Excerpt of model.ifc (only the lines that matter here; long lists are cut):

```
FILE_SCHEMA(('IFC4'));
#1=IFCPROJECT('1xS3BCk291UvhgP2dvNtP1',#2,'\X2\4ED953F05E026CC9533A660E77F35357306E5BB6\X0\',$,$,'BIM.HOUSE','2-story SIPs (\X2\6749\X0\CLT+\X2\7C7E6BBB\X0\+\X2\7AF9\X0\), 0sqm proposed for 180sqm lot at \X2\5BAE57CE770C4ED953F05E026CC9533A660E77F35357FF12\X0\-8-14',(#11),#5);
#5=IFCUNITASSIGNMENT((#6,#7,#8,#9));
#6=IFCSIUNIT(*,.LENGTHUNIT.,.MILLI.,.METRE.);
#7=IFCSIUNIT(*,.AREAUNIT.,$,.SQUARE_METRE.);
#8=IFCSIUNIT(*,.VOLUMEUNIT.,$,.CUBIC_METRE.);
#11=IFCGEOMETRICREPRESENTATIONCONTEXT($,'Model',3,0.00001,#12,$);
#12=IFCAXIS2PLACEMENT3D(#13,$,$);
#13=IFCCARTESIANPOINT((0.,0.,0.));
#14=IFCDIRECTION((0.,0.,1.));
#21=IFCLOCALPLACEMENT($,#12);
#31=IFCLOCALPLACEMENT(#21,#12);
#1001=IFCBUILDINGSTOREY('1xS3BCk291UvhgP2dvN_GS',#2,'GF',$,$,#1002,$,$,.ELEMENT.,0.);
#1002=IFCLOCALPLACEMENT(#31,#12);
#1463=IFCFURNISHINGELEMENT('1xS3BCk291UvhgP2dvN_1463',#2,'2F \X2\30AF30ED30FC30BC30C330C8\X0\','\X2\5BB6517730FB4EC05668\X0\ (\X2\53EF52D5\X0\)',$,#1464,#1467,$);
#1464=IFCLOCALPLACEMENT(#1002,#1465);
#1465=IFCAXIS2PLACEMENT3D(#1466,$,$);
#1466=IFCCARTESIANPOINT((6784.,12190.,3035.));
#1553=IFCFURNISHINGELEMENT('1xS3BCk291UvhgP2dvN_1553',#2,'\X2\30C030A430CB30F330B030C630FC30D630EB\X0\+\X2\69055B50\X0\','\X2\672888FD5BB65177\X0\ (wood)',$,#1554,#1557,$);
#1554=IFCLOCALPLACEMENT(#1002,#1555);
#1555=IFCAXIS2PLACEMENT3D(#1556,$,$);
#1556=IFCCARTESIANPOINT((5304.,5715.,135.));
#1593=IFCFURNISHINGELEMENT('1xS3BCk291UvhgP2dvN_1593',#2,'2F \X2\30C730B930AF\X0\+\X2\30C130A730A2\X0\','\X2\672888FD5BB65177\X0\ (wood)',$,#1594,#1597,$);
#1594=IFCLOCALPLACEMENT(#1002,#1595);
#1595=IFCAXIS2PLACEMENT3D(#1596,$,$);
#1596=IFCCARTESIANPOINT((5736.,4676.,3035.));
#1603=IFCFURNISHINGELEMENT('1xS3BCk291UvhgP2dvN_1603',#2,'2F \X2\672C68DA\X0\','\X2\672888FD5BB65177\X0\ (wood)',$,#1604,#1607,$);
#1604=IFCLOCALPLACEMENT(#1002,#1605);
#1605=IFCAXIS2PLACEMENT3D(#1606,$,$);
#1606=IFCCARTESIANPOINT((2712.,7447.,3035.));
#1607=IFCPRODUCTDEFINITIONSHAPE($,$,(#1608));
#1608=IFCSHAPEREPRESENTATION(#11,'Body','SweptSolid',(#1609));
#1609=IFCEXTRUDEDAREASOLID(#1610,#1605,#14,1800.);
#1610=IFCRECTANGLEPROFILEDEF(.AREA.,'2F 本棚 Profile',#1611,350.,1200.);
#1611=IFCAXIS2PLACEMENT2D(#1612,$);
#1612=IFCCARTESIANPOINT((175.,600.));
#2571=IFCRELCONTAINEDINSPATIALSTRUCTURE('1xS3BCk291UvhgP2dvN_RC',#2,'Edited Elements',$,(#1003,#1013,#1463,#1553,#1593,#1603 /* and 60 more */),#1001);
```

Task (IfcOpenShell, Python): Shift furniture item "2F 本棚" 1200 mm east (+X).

```python
import ifcopenshell
import ifcopenshell.api.geometry
import ifcopenshell.util.placement
import ifcopenshell.util.unit

model = ifcopenshell.open("model.ifc")
unit_scale = ifcopenshell.util.unit.calculate_unit_scale(model)

item = model.by_guid("1xS3BCk291UvhgP2dvN_1603")
matrix = ifcopenshell.util.placement.get_local_placement(item.ObjectPlacement)
matrix[0, 3] += 1.2 / unit_scale
ifcopenshell.api.geometry.edit_object_placement(model, product=item, matrix=matrix, is_si=False)

print(ifcopenshell.util.placement.get_local_placement(item.ObjectPlacement).round(3) + 0.0)

model.write("model_updated.ifc")
```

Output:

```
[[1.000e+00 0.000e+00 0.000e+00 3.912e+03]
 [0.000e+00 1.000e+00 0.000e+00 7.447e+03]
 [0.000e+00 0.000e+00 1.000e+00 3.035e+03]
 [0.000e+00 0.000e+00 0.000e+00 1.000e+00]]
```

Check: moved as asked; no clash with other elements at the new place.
